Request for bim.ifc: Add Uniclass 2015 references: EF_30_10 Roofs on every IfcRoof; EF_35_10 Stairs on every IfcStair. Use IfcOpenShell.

First a look at what the model holds.

```python
import ifcopenshell

model = ifcopenshell.open("bim.ifc")
print(model.schema)
print("classifications:", [c.Name for c in model.by_type("IfcClassification")])
for ifc_class in ("IfcDoor", "IfcRoof", "IfcStair", "IfcWall", "IfcWindow"):
    print(ifc_class, len(model.by_type(ifc_class)))
```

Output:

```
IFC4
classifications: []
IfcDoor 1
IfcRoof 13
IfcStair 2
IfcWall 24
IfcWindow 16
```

```python
import ifcopenshell
import ifcopenshell.api.classification

model = ifcopenshell.open("bim.ifc")

system = ifcopenshell.api.classification.add_classification(model, classification="Uniclass 2015")

codes = {
    "IfcRoof": ("EF_30_10", "Roofs"),
    "IfcStair": ("EF_35_10", "Stairs"),
}
for ifc_class, (code, name) in codes.items():
    products = model.by_type(ifc_class)
    ifcopenshell.api.classification.add_reference(
        model, products=products, classification=system, identification=code, name=name
    )
    print(code, len(products))

model.write("bim_updated.ifc")
```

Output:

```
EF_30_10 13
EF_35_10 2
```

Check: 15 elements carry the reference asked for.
